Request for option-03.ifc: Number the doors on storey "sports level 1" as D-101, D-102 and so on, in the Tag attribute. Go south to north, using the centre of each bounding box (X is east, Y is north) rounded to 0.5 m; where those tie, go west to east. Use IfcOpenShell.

First a look at what the model holds.

```python
import ifcopenshell
import ifcopenshell.util.element
import ifcopenshell.util.placement

model = ifcopenshell.open("option-03.ifc")
print(model.schema)
storey = next(s for s in model.by_type("IfcBuildingStorey") if s.Name == "sports level 1")
doors = [e for e in ifcopenshell.util.element.get_decomposition(storey) if e.is_a("IfcDoor")]
for e in sorted(doors, key=lambda e: e.id()):
    origin = ifcopenshell.util.placement.get_local_placement(e.ObjectPlacement)[:3, 3]
    print(e.id(), e.Tag, e.Name, origin.round(2) + 0.0, sep=" | ")
```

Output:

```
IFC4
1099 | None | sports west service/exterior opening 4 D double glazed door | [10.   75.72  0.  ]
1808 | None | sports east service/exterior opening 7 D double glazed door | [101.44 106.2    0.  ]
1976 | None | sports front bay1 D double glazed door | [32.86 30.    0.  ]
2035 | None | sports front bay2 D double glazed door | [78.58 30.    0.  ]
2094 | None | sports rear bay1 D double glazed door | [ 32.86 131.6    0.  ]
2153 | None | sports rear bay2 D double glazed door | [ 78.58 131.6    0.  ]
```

```python
import ifcopenshell
import ifcopenshell.geom
import ifcopenshell.util.element
import ifcopenshell.util.shape

model = ifcopenshell.open("option-03.ifc")
settings = ifcopenshell.geom.settings()
settings.set("use-world-coords", True)


def centre(element):
    shape = ifcopenshell.geom.create_shape(settings, element)
    return ifcopenshell.util.shape.get_bbox_centroid(shape.geometry)


storey = next(s for s in model.by_type("IfcBuildingStorey") if s.Name == "sports level 1")
doors = [e for e in ifcopenshell.util.element.get_decomposition(storey) if e.is_a("IfcDoor")]

# Insertion points can sit at a corner or the storey origin, so sort by the geometry (in metres).
centres = {e: centre(e) for e in doors}
doors.sort(key=lambda e: (round(centres[e][1] / 0.5), centres[e][0]))

for i, e in enumerate(doors, start=1):
    number = f"D-1{i:02d}"
    e.Tag = number
    print(e.id(), number)

model.write("option-03_updated.ifc")
```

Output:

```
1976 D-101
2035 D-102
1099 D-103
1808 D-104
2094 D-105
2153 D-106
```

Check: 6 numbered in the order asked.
